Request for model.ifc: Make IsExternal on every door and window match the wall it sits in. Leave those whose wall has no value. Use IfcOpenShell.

First a look at what the model holds.

```python
import ifcopenshell
import ifcopenshell.util.element

model = ifcopenshell.open("model.ifc")
print(model.schema)
seen = {}
for e in model.by_type("IfcDoor") + model.by_type("IfcWindow"):
    if not e.FillsVoids:
        continue
    host = e.FillsVoids[0].RelatingOpeningElement.VoidsElements[0].RelatingBuildingElement
    own = ifcopenshell.util.element.get_pset(e, f"Pset_{e.is_a()[3:].removesuffix('StandardCase')}Common", "IsExternal")
    wall = ifcopenshell.util.element.get_pset(host, "Pset_WallCommon", "IsExternal")
    seen[e.is_a(), own, wall] = seen.get((e.is_a(), own, wall), 0) + 1
for (cls, own, wall), count in sorted(seen.items(), key=str):
    print(count, cls, "IsExternal:", own, "| host wall:", wall)
```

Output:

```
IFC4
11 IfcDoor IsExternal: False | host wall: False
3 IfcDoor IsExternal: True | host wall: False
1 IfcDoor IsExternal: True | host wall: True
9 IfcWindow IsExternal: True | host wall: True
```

```python
import ifcopenshell
import ifcopenshell.api.pset
import ifcopenshell.util.element

model = ifcopenshell.open("model.ifc")

count = 0
for ifc_class, pset_name in (("IfcDoor", "Pset_DoorCommon"), ("IfcWindow", "Pset_WindowCommon")):
    for e in model.by_type(ifc_class):
        if not e.FillsVoids:
            continue
        host = e.FillsVoids[0].RelatingOpeningElement.VoidsElements[0].RelatingBuildingElement
        external = ifcopenshell.util.element.get_pset(host, "Pset_WallCommon", "IsExternal")
        if external is None or ifcopenshell.util.element.get_pset(e, pset_name, "IsExternal") == external:
            continue
        pset = ifcopenshell.api.pset.add_pset(model, product=e, name=pset_name)
        ifcopenshell.api.pset.edit_pset(model, pset=pset, properties={"IsExternal": external})
        count += 1

print(count, "updated")

model.write("model_rev.ifc")
```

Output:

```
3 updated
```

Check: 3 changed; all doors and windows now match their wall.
